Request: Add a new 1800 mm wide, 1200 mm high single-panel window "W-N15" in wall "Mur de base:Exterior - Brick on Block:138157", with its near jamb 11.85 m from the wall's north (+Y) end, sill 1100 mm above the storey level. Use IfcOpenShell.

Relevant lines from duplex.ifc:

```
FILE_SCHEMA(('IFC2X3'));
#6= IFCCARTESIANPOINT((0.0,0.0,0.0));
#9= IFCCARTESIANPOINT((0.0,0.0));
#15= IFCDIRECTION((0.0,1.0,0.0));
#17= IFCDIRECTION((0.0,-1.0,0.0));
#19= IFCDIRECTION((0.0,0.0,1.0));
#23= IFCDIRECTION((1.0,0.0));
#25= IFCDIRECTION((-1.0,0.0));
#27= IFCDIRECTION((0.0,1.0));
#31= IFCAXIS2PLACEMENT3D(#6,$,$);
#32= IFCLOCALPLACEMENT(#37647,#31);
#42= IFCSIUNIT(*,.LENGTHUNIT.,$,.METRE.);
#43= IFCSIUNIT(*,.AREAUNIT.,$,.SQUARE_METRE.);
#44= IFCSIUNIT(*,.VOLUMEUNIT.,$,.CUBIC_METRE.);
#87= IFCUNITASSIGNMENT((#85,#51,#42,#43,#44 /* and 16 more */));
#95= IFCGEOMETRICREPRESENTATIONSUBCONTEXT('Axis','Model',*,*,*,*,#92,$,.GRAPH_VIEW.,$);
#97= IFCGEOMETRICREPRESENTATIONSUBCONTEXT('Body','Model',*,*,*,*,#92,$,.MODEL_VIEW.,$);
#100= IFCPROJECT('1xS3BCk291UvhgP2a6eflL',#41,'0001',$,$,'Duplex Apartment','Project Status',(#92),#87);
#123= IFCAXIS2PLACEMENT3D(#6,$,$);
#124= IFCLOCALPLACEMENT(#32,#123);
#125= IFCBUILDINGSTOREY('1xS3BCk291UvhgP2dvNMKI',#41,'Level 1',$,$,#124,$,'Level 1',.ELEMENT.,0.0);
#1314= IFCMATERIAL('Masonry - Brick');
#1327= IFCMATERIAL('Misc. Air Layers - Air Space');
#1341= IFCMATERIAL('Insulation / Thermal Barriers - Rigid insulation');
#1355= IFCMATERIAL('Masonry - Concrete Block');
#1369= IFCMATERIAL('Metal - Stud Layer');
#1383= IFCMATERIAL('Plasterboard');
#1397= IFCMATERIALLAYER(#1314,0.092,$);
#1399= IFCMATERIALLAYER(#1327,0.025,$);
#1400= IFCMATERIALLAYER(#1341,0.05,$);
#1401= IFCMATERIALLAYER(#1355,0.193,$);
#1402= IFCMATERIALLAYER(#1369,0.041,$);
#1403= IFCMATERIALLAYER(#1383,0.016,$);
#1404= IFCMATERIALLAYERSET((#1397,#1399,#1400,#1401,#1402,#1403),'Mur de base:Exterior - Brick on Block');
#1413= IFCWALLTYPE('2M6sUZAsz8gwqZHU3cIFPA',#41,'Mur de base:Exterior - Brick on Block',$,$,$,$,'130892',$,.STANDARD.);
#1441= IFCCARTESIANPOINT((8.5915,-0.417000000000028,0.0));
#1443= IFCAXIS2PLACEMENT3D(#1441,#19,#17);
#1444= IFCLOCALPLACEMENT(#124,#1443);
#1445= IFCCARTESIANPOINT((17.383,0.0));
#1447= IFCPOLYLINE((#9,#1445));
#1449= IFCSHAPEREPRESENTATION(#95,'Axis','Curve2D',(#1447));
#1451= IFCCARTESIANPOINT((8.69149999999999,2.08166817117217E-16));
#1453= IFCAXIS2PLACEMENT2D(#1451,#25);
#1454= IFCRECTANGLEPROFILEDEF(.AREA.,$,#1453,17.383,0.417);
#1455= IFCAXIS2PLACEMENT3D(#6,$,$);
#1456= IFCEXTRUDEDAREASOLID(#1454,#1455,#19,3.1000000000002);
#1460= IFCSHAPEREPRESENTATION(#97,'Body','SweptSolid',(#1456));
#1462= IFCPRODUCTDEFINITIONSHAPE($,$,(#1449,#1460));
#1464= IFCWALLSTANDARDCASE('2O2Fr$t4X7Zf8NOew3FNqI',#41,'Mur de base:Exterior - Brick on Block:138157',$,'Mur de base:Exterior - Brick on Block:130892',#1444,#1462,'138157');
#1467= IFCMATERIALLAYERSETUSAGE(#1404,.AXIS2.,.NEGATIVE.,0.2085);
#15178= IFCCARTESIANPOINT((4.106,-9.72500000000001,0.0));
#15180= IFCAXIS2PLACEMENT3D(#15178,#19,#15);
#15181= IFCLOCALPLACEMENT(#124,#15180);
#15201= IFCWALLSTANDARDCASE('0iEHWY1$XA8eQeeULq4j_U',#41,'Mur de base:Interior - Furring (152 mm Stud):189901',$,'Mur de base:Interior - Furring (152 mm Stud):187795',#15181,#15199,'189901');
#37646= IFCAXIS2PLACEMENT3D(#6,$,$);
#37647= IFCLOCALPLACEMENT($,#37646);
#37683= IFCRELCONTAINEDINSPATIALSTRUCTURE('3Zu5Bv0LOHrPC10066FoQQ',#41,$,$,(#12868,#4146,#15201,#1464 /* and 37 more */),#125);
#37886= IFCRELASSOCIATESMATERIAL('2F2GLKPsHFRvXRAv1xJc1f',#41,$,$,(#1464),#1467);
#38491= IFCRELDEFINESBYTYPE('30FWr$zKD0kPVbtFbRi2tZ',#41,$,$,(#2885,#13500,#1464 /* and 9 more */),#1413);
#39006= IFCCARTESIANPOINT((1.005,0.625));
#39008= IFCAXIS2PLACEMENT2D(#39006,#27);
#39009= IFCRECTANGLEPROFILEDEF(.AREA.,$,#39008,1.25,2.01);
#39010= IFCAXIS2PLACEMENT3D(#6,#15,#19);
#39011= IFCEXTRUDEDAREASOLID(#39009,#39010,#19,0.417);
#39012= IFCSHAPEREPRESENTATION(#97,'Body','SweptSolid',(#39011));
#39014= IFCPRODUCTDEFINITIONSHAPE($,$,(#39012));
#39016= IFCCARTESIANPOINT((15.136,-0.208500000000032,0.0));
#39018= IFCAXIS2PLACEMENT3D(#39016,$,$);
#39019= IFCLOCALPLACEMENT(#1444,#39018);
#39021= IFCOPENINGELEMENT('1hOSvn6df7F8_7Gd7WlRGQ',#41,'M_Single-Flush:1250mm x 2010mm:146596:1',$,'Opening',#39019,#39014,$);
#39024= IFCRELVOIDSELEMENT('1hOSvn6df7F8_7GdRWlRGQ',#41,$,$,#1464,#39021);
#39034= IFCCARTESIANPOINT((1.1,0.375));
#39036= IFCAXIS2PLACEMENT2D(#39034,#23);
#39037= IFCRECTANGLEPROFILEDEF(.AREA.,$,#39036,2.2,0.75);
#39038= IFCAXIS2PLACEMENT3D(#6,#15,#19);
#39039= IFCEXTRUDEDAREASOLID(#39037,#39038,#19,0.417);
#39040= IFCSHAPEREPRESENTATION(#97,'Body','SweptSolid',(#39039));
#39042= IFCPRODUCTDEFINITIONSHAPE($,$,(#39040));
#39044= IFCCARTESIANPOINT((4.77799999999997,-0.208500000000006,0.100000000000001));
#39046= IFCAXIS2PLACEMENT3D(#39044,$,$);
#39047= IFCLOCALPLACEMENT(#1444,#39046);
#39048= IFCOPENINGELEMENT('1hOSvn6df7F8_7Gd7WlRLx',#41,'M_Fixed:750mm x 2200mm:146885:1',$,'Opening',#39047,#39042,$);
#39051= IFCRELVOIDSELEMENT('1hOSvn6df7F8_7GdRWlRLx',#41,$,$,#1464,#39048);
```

```python
import numpy as np
import ifcopenshell
import ifcopenshell.api.feature
import ifcopenshell.api.geometry
import ifcopenshell.api.root
import ifcopenshell.api.spatial
import ifcopenshell.api.type
import ifcopenshell.geom
import ifcopenshell.util.element
import ifcopenshell.util.placement
import ifcopenshell.util.representation
import ifcopenshell.util.shape
import ifcopenshell.util.unit

model = ifcopenshell.open("duplex.ifc")
unit_scale = ifcopenshell.util.unit.calculate_unit_scale(model)
settings = ifcopenshell.geom.settings()


def volume(element):
    """Net volume in cubic metres, openings subtracted."""
    shape = ifcopenshell.geom.create_shape(settings, element)
    return ifcopenshell.util.shape.get_volume(shape.geometry)


wall = model.by_guid("2O2Fr$t4X7Zf8NOew3FNqI")
storey = ifcopenshell.util.element.get_container(wall, ifc_class="IfcBuildingStorey")
context = ifcopenshell.util.representation.get_context(model, "Model", "Body", "MODEL_VIEW")
before = volume(wall)

width, height, from_end, sill = 1.8, 1.2, 11.85, 1.1  # metres

# The wall runs along its own X axis, and the end named is its -X end.
wall_shape = ifcopenshell.geom.create_shape(settings, wall)
x, y, z = ifcopenshell.util.shape.get_vertices(wall_shape.geometry).T
start = x.min() + from_end
face, thickness = float(y.min()), float(y.max() - y.min())
wall_matrix = ifcopenshell.util.placement.get_local_placement(wall.ObjectPlacement)
level = ifcopenshell.util.placement.get_local_placement(storey.ObjectPlacement)[2, 3]


def in_wall(x, y):
    """Placement at x, y metres in the wall's axes, at sill height."""
    matrix = wall_matrix.copy()
    matrix[:, 3] = wall_matrix @ np.array([x / unit_scale, y / unit_scale, 0.0, 1.0])
    matrix[2, 3] = level + sill / unit_scale
    return matrix


# Opening: a box that overshoots both wall faces by 50 mm.
opening = ifcopenshell.api.root.create_entity(model, ifc_class="IfcOpeningElement")
box = ifcopenshell.api.geometry.add_wall_representation(
    model, context=context, length=width, height=height, thickness=thickness + 0.1
)
ifcopenshell.api.geometry.assign_representation(model, product=opening, representation=box)
ifcopenshell.api.geometry.edit_object_placement(model, product=opening, matrix=in_wall(start, face - 0.05), is_si=False)
ifcopenshell.api.feature.add_feature(model, feature=opening, element=wall)

window = ifcopenshell.api.root.create_entity(model, ifc_class="IfcWindow", name="W-N15")
window.OverallWidth, window.OverallHeight = width / unit_scale, height / unit_scale
body = ifcopenshell.api.geometry.add_window_representation(
    model,
    context=context,
    overall_width=window.OverallWidth,
    overall_height=window.OverallHeight,
    partition_type="SINGLE_PANEL",
)
ifcopenshell.api.geometry.assign_representation(model, product=window, representation=body)
ifcopenshell.api.spatial.assign_container(model, products=[window], relating_structure=storey)
fills = ifcopenshell.api.feature.add_filling(model, opening=opening, element=window)
fills.OwnerHistory = window.OwnerHistory  # required in IFC2X3

# IFC2X3 keeps the operation on the window style.
style = ifcopenshell.api.root.create_entity(model, ifc_class="IfcWindowStyle", name="W-N15")
style.OperationType, style.ConstructionType = "SINGLE_PANEL", "NOTDEFINED"
style.ParameterTakesPrecedence = style.Sizeable = False
ifcopenshell.api.type.assign_type(model, related_objects=[window], relating_type=style)

# Centre the window in the wall's thickness.
ifcopenshell.api.geometry.edit_object_placement(model, product=window, matrix=in_wall(start, face), is_si=False)
window_shape = ifcopenshell.geom.create_shape(settings, window)
depth = ifcopenshell.util.shape.get_vertices(window_shape.geometry)[:, 1]
offset = face + thickness / 2 - (depth.min() + depth.max()) / 2
ifcopenshell.api.geometry.edit_object_placement(model, product=window, matrix=in_wall(start, offset), is_si=False)

after = volume(wall)

print(f"wall volume {before:.3f} -> {after:.3f} m3")

model.write("duplex_v2.ifc")
```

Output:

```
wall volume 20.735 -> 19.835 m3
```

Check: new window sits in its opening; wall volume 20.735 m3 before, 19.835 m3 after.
